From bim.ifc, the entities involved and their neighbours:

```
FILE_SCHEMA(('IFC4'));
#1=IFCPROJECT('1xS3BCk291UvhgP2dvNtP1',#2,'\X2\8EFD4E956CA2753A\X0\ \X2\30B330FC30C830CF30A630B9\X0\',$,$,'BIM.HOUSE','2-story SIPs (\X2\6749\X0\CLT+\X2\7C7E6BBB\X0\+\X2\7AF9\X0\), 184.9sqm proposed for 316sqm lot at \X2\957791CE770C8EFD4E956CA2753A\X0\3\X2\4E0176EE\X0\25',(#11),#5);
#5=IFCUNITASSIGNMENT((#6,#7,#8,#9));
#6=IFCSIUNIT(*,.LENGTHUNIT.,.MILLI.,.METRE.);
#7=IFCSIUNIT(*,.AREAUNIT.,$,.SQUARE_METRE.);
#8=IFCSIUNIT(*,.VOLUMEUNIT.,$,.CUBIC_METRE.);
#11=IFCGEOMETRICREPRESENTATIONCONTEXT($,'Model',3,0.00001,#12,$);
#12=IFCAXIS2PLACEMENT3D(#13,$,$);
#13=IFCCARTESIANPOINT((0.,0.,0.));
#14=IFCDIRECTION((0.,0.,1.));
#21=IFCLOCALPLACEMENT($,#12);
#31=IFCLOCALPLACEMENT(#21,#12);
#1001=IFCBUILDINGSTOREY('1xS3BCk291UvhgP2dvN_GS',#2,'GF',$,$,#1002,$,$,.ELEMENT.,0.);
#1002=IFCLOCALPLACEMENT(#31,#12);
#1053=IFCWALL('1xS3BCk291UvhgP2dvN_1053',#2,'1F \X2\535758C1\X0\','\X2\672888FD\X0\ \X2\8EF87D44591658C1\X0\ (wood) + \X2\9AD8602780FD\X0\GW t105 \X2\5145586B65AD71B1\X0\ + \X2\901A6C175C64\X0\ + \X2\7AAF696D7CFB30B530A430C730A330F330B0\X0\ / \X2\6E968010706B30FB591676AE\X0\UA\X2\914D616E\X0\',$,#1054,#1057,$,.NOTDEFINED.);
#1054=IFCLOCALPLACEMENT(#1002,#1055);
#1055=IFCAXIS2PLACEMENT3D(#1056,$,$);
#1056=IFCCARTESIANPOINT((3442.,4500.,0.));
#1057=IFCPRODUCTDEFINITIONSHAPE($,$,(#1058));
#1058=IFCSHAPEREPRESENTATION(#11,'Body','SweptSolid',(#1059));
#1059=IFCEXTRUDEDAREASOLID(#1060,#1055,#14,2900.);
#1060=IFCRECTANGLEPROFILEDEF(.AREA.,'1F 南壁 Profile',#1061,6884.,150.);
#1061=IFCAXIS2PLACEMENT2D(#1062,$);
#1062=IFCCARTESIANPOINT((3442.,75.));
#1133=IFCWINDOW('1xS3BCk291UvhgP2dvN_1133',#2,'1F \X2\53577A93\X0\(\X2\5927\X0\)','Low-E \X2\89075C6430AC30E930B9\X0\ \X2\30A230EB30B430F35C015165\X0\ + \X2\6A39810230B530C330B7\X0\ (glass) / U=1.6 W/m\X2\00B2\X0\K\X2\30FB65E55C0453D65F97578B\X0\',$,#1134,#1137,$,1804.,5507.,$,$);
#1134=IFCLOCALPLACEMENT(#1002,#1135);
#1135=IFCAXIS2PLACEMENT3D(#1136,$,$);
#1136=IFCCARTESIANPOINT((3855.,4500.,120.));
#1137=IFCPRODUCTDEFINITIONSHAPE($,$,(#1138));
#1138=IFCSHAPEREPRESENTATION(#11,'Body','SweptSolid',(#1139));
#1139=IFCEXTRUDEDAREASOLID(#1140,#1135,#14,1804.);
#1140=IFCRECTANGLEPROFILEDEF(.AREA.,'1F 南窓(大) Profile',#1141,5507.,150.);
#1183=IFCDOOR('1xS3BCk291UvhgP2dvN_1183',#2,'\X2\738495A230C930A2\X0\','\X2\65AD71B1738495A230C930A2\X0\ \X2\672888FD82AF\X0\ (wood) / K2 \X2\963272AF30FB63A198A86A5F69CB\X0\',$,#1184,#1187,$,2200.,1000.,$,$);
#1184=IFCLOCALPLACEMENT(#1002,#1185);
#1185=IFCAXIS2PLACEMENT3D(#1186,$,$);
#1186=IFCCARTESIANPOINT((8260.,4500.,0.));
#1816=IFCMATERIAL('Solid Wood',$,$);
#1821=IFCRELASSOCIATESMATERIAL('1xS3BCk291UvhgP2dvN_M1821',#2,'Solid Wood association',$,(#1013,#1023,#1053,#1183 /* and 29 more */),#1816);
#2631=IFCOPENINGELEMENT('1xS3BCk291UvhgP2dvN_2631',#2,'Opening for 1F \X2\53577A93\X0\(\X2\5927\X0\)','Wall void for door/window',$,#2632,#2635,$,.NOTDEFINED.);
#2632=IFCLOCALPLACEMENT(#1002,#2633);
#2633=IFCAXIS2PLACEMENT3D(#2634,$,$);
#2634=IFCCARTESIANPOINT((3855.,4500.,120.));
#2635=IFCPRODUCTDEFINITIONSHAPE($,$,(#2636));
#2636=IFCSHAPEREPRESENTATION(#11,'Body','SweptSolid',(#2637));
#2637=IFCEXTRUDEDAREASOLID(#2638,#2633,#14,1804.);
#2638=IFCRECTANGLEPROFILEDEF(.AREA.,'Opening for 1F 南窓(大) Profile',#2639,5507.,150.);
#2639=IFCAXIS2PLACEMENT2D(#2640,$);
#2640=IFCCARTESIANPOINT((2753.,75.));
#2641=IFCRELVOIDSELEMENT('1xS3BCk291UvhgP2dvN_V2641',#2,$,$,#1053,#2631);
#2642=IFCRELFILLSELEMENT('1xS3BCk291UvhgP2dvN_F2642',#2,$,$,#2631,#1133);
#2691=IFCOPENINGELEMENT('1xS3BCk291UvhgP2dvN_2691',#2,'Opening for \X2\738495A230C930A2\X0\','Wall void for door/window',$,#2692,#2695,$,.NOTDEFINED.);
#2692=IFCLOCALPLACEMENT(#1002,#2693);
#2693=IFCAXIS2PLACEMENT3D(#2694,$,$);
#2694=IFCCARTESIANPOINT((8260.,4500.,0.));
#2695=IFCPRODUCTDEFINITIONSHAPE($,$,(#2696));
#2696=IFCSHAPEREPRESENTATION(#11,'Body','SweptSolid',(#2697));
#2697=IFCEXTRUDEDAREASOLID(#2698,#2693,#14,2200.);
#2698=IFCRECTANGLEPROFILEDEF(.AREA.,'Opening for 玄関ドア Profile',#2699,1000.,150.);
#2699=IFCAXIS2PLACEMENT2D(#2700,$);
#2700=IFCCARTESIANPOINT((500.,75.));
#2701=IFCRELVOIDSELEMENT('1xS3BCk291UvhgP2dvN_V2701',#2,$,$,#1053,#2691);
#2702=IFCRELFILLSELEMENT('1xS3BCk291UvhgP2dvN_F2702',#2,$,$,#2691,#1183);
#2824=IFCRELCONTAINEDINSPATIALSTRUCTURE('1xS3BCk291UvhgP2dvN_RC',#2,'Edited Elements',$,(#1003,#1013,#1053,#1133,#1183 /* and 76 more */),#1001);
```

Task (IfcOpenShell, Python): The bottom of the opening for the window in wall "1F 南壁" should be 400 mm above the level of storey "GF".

```python
import numpy as np
import ifcopenshell
import ifcopenshell.api.geometry
import ifcopenshell.geom
import ifcopenshell.util.element
import ifcopenshell.util.placement
import ifcopenshell.util.shape
import ifcopenshell.util.unit

model = ifcopenshell.open("bim.ifc")
unit_scale = ifcopenshell.util.unit.calculate_unit_scale(model)

window = model.by_id(1133)
opening = window.FillsVoids[0].RelatingOpeningElement
storey = ifcopenshell.util.element.get_container(window, ifc_class="IfcBuildingStorey")
level = ifcopenshell.util.placement.get_local_placement(storey.ObjectPlacement)[2, 3]

# The opening's origin need not be at the sill, so measure its lowest point.
shape = ifcopenshell.geom.create_shape(ifcopenshell.geom.settings(), opening)
bottom = ifcopenshell.util.shape.get_shape_bottom_elevation(shape, shape.geometry) / unit_scale
dz = level + 0.4 / unit_scale - bottom

shift = np.array([0.0, 0.0, dz])
# The window is not placed relative to its opening, so move both.
for product in (opening, window):
    matrix = ifcopenshell.util.placement.get_local_placement(product.ObjectPlacement)
    matrix[:3, 3] += shift
    ifcopenshell.api.geometry.edit_object_placement(model, product=product, matrix=matrix, is_si=False)

print(f"moved by {dz * unit_scale:+.3f} m")

model.write("bim-out.ifc")
```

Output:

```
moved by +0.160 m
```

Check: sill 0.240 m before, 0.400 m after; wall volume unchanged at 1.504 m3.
